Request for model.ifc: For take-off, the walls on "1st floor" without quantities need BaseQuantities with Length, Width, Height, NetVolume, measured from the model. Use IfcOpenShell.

First a look at what the model holds.

```python
import ifcopenshell
import ifcopenshell.util.element
import ifcopenshell.util.unit

model = ifcopenshell.open("model.ifc")
print(model.schema)
for unit_type in ("LENGTHUNIT", "AREAUNIT", "VOLUMEUNIT"):
    print(unit_type, ifcopenshell.util.unit.calculate_unit_scale(model, unit_type))
storey = next(s for s in model.by_type("IfcBuildingStorey") if s.Name == "1st floor")
walls = [e for e in ifcopenshell.util.element.get_decomposition(storey) if e.is_a("IfcWall")]
for e in sorted(walls, key=lambda e: e.id()):
    print(e.id(), e.is_a(), e.Name, list(ifcopenshell.util.element.get_psets(e, qtos_only=True)), sep=" | ")
```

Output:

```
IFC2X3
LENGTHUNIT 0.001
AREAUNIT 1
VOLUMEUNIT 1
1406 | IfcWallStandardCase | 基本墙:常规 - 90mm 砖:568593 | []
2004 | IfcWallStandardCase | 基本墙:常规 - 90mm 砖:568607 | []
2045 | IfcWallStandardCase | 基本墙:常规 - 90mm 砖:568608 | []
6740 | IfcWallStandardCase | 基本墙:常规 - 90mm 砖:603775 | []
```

```python
import ifcopenshell
import ifcopenshell.api.pset
import ifcopenshell.geom
import ifcopenshell.util.element
import ifcopenshell.util.shape
import ifcopenshell.util.unit

model = ifcopenshell.open("model.ifc")
unit_scale = ifcopenshell.util.unit.calculate_unit_scale(model)
volume_scale = ifcopenshell.util.unit.calculate_unit_scale(model, "VOLUMEUNIT")
settings = ifcopenshell.geom.settings()

storey = next(s for s in model.by_type("IfcBuildingStorey") if s.Name == "1st floor")
walls = [e for e in ifcopenshell.util.element.get_decomposition(storey) if e.is_a("IfcWall")]

for e in sorted(walls, key=lambda e: e.id()):
    if ifcopenshell.util.element.get_psets(e, qtos_only=True, should_inherit=False):
        continue
    # Geometry comes back in metres, in the element's own axes.
    shape = ifcopenshell.geom.create_shape(settings, e)
    values = {
        "Length": ifcopenshell.util.shape.get_x(shape.geometry) / unit_scale,
        "Width": ifcopenshell.util.shape.get_y(shape.geometry) / unit_scale,
        "Height": ifcopenshell.util.shape.get_z(shape.geometry) / unit_scale,
        "NetVolume": ifcopenshell.util.shape.get_volume(shape.geometry) / volume_scale,
    }
    qto = ifcopenshell.api.pset.add_qto(model, product=e, name="BaseQuantities")
    ifcopenshell.api.pset.edit_qto(model, qto=qto, properties=values)
    print(e.id(), {k: round(v, 3) for k, v in values.items()})

model.write("model-out.ifc")
```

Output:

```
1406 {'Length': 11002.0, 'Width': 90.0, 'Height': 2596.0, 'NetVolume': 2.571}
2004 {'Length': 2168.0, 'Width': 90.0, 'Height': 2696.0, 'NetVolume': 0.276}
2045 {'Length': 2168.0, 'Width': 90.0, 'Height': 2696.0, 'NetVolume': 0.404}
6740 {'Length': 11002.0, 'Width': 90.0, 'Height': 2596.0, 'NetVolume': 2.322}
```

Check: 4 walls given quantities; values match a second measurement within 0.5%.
